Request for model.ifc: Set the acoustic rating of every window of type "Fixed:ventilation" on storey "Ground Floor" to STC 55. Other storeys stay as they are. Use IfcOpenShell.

First a look at what the model holds.

```python
import ifcopenshell
import ifcopenshell.util.element

model = ifcopenshell.open("model.ifc")
print(model.schema)
storey = next(s for s in model.by_type("IfcBuildingStorey") if s.Name == "Ground Floor")
windows = [e for e in ifcopenshell.util.element.get_decomposition(storey) if e.is_a("IfcWindow")]
seen = {}
for e in windows:
    element_type = ifcopenshell.util.element.get_type(e)
    key = (element_type.Name if element_type != e and element_type else None, ifcopenshell.util.element.get_pset(e, "Pset_WindowCommon", "AcousticRating"))
    seen[key] = seen.get(key, 0) + 1
for (name, value), count in sorted(seen.items(), key=str):
    print(count, "x", name, "|", value)
```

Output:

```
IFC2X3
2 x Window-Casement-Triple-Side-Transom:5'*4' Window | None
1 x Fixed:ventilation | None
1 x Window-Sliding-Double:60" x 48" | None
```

```python
import ifcopenshell
import ifcopenshell.api.pset
import ifcopenshell.util.element

model = ifcopenshell.open("model.ifc")

storey = next(s for s in model.by_type("IfcBuildingStorey") if s.Name == "Ground Floor")
windows = [e for e in ifcopenshell.util.element.get_decomposition(storey) if e.is_a("IfcWindow")]

count = 0
for e in windows:
    element_type = ifcopenshell.util.element.get_type(e)
    if element_type in (None, e) or element_type.Name != "Fixed:ventilation":
        continue
    # add_pset returns the element's existing set when there is one.
    pset = ifcopenshell.api.pset.add_pset(model, product=e, name="Pset_WindowCommon")
    ifcopenshell.api.pset.edit_pset(model, pset=pset, properties={"AcousticRating": "STC 55"})
    count += 1

print(count, "windows updated")

model.write("model_v2.ifc")
```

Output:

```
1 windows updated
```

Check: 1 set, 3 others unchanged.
